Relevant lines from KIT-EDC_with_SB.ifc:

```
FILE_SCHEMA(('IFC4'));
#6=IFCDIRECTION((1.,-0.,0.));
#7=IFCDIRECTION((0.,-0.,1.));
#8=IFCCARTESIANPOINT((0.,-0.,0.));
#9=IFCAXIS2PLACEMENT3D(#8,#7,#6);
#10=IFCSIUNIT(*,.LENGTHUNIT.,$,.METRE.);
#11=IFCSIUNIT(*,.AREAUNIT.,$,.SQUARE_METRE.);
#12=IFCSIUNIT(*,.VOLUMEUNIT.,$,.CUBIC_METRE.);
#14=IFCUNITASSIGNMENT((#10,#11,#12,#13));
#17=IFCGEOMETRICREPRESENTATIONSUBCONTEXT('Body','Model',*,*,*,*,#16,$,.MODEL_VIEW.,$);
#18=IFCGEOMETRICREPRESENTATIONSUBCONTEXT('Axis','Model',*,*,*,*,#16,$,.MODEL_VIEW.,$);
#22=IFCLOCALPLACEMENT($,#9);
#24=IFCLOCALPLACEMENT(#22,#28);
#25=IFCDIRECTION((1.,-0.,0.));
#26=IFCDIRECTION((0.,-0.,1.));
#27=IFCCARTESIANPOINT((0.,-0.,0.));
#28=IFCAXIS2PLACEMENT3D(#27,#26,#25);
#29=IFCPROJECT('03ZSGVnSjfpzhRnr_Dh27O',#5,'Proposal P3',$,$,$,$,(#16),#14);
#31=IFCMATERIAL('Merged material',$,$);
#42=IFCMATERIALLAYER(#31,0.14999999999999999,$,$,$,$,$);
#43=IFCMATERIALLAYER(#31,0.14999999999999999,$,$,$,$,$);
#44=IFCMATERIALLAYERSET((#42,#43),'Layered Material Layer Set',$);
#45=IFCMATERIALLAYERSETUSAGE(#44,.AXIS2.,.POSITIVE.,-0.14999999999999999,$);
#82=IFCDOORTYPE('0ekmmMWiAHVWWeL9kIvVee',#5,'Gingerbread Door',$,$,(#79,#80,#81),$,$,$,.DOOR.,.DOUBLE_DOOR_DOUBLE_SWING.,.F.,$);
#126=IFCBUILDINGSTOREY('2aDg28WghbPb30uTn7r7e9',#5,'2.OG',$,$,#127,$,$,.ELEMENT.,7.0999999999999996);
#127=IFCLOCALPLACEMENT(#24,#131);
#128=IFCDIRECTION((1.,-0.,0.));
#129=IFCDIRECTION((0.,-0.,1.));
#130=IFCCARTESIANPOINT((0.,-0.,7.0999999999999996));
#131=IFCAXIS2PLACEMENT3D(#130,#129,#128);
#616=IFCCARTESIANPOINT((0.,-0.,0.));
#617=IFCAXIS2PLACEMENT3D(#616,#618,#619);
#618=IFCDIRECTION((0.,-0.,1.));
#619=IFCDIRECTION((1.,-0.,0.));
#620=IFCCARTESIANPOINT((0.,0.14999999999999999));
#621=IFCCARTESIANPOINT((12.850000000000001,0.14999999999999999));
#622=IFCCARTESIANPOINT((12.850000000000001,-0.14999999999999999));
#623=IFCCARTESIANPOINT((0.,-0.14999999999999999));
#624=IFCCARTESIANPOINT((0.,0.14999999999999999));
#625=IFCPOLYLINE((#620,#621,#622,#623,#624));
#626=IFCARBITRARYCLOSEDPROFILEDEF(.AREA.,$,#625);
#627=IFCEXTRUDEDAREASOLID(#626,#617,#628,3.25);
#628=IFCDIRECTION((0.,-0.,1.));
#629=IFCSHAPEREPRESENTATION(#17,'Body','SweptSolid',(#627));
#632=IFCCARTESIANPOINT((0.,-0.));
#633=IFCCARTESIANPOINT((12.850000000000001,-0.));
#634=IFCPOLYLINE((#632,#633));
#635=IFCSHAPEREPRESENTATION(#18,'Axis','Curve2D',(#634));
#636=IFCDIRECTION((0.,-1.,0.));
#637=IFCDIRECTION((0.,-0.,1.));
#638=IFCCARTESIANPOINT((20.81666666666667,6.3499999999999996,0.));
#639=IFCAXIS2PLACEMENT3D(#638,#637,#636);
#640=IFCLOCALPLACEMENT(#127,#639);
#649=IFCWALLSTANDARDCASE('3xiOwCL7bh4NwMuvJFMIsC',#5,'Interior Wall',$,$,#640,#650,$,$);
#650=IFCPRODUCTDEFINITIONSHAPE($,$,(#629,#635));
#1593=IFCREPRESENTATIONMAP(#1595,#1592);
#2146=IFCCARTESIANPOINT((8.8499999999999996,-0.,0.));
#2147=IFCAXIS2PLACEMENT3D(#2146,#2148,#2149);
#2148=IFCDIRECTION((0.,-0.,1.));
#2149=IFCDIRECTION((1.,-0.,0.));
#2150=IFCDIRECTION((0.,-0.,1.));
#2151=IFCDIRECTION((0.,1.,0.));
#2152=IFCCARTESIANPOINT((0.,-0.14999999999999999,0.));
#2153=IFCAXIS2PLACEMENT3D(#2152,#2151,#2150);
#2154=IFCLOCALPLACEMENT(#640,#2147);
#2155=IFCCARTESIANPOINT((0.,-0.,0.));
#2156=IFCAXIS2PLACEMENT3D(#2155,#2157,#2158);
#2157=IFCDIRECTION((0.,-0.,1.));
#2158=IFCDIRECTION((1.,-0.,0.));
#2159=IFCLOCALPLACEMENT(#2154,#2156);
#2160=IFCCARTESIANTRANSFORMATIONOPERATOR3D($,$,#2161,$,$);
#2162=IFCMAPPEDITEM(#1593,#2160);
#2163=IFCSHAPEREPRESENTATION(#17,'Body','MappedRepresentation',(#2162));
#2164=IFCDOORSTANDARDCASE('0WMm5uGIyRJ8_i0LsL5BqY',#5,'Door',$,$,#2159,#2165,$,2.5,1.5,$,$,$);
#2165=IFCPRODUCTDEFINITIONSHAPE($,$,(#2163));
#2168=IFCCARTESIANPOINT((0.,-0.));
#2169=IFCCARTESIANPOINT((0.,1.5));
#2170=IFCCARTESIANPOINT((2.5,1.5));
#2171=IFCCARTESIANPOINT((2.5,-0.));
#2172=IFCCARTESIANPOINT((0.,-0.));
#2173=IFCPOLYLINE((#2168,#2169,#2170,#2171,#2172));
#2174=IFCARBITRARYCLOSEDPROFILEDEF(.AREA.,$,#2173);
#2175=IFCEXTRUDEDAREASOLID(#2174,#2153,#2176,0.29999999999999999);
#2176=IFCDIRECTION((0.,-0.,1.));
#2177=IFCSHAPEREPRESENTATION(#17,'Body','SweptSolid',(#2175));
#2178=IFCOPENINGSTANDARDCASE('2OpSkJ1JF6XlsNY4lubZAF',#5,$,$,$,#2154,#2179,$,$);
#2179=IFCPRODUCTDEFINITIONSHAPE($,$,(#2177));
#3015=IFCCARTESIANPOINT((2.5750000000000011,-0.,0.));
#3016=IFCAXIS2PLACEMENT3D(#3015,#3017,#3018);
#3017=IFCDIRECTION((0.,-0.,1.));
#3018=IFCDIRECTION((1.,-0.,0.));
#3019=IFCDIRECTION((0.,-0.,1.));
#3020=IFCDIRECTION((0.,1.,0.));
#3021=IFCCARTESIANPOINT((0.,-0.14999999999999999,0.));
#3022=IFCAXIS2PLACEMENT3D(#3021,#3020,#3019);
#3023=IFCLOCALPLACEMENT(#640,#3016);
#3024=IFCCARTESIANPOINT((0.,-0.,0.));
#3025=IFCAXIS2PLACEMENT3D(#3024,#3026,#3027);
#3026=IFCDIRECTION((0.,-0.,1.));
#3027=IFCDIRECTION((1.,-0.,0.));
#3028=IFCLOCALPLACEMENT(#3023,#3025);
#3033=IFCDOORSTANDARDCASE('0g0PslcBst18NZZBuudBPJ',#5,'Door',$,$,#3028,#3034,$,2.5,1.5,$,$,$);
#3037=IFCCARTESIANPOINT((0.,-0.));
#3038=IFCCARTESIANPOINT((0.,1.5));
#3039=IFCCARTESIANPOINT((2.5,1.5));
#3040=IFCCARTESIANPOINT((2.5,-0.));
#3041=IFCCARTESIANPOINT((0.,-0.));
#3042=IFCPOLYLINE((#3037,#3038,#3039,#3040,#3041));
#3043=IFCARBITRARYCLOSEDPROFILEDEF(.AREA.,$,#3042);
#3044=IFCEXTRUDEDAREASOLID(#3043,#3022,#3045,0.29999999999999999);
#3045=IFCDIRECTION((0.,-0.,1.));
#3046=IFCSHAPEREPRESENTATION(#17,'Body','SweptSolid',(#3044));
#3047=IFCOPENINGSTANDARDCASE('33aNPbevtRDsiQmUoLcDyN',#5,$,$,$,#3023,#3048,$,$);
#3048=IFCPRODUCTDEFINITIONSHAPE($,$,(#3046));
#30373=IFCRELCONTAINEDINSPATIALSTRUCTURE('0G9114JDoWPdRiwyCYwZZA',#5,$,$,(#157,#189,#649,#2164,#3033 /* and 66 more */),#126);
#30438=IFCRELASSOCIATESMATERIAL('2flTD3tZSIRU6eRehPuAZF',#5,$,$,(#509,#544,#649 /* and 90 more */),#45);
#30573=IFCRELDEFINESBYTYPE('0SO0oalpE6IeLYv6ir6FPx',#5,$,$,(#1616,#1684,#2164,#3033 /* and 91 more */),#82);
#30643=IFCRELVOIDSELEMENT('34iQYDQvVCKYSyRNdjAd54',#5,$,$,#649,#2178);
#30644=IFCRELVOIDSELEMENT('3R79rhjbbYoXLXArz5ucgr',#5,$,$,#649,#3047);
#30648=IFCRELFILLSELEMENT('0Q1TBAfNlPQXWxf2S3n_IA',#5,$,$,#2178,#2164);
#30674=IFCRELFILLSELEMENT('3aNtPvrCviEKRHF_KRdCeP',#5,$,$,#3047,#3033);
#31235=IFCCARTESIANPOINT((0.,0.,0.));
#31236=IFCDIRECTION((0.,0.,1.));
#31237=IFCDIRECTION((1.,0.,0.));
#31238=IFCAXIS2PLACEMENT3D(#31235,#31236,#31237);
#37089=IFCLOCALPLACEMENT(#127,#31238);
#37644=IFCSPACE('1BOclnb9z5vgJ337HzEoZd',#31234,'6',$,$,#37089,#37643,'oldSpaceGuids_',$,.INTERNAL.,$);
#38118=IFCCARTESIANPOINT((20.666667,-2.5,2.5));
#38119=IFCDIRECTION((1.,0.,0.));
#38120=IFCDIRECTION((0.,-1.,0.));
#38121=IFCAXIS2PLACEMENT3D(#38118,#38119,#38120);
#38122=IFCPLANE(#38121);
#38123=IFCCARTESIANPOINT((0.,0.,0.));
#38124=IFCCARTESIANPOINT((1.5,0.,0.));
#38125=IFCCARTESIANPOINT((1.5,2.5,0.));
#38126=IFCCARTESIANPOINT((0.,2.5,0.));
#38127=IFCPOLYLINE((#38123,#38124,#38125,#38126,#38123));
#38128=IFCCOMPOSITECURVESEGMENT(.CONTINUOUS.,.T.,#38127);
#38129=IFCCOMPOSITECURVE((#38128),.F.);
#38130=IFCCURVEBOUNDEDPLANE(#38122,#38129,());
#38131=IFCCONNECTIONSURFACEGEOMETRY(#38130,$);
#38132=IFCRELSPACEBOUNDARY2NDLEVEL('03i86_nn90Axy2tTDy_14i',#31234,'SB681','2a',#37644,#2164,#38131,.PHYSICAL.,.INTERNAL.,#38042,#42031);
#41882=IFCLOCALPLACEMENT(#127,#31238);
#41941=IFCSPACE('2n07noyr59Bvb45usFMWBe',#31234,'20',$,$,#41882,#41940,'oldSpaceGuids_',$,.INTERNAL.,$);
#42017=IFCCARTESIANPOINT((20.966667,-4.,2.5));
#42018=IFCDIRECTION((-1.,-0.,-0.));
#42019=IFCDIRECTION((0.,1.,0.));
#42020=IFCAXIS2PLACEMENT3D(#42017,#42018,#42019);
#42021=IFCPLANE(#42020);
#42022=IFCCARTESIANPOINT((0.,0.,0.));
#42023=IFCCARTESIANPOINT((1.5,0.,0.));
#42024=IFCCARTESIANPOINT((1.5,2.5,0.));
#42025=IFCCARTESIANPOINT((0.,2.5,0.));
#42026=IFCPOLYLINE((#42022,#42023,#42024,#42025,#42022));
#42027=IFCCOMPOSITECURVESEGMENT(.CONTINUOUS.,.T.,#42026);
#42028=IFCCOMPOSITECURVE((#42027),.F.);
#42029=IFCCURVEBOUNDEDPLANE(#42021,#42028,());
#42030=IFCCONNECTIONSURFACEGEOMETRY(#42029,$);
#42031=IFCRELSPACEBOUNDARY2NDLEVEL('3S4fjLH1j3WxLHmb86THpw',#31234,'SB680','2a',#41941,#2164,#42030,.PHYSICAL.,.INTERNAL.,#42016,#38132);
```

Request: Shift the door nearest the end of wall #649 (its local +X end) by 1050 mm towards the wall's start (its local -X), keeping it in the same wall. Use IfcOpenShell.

```python
import numpy as np
import ifcopenshell
import ifcopenshell.api.geometry
import ifcopenshell.util.placement

model = ifcopenshell.open("KIT-EDC_with_SB.ifc")

door = model.by_guid("0WMm5uGIyRJ8_i0LsL5BqY")
opening = door.FillsVoids[0].RelatingOpeningElement
wall = opening.VoidsElements[0].RelatingBuildingElement

wall_matrix = ifcopenshell.util.placement.get_local_placement(wall.ObjectPlacement)
shift = wall_matrix[:3, 0] * -1.05
before = ifcopenshell.util.placement.get_local_placement(door.ObjectPlacement)[:3, 3].copy()

# The door is placed relative to its opening, so it follows when the opening moves.
matrix = ifcopenshell.util.placement.get_local_placement(opening.ObjectPlacement)
matrix[:3, 3] += shift
ifcopenshell.api.geometry.edit_object_placement(
    model, product=opening, matrix=matrix, is_si=False, should_transform_children=True
)

# Space boundary surfaces are stored in each space's coordinates; move them too.
for rel in door.ProvidesBoundaries:
    if not rel.ConnectionGeometry:
        continue
    surface = rel.ConnectionGeometry.SurfaceOnRelatingElement.BasisSurface
    space_matrix = ifcopenshell.util.placement.get_local_placement(rel.RelatingSpace.ObjectPlacement)
    point = np.array(surface.Position.Location.Coordinates) + space_matrix[:3, :3].T @ shift
    surface.Position = model.createIfcAxis2Placement3D(
        model.createIfcCartesianPoint(point.tolist()), surface.Position.Axis, surface.Position.RefDirection
    )

after = ifcopenshell.util.placement.get_local_placement(door.ObjectPlacement)[:3, 3]
print("door moved by", (after - before).round(3) + 0.0)

model.write("KIT-EDC_with_SB_v2.ifc")
```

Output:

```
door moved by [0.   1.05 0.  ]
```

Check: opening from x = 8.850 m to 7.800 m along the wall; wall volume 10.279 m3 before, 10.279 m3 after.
